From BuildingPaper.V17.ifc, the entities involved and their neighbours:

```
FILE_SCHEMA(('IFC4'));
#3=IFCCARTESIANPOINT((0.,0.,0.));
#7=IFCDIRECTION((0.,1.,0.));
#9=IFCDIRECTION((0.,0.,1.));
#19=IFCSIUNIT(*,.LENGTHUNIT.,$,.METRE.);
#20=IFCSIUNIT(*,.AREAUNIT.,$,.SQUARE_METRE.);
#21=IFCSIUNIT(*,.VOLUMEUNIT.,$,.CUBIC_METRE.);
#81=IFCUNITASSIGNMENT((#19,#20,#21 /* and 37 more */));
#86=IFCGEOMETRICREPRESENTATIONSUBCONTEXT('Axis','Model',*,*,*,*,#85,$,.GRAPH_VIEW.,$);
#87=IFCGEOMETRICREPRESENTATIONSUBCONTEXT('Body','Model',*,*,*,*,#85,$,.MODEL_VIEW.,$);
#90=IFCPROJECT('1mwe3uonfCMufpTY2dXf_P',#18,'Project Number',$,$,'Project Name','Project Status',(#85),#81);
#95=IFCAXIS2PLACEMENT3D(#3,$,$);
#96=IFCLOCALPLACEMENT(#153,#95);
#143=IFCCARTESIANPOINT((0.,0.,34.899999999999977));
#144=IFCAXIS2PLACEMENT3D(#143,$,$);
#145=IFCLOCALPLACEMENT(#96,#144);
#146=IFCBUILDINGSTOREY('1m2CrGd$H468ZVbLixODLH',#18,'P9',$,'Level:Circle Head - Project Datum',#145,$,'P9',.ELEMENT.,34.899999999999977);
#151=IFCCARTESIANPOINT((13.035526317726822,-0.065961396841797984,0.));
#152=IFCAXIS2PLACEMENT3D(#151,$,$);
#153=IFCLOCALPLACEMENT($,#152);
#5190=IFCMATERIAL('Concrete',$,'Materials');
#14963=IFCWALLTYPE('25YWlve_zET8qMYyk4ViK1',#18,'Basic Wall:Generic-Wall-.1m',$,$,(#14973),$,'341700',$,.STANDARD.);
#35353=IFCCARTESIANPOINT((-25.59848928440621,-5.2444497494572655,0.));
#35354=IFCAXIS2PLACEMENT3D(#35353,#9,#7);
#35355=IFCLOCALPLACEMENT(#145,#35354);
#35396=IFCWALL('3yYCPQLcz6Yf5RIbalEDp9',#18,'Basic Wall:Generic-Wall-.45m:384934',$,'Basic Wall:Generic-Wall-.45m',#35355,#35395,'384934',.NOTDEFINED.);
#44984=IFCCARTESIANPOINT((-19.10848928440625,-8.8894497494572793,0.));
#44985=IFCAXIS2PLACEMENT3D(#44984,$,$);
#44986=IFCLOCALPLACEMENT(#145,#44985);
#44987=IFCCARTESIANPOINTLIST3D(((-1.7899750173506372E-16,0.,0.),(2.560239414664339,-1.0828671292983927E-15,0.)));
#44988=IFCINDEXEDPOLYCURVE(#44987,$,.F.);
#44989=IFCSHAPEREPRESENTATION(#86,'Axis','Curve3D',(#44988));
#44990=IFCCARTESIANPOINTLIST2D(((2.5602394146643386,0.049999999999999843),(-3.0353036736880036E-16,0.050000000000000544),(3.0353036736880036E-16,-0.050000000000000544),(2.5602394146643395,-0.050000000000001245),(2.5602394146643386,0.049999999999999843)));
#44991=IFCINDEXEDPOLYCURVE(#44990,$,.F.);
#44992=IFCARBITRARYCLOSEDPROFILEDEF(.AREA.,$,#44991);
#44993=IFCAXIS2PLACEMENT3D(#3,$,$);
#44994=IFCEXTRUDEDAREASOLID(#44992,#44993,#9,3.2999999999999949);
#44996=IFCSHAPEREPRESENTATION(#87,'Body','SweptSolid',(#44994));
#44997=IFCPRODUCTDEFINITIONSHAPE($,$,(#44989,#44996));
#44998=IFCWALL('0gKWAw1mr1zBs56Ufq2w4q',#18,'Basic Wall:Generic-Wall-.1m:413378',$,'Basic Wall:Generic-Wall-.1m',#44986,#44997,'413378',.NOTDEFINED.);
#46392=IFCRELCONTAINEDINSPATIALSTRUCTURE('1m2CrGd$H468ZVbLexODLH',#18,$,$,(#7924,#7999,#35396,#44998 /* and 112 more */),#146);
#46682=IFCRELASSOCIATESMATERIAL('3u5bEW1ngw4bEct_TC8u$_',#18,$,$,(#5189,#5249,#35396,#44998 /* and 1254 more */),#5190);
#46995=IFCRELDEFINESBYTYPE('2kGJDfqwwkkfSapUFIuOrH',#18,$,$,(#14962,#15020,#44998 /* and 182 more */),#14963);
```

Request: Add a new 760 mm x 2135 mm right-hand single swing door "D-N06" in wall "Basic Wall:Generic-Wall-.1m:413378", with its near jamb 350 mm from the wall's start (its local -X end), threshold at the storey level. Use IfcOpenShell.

```python
import numpy as np
import ifcopenshell
import ifcopenshell.api.feature
import ifcopenshell.api.geometry
import ifcopenshell.api.root
import ifcopenshell.api.spatial
import ifcopenshell.geom
import ifcopenshell.util.element
import ifcopenshell.util.placement
import ifcopenshell.util.representation
import ifcopenshell.util.shape
import ifcopenshell.util.unit

model = ifcopenshell.open("BuildingPaper.V17.ifc")
unit_scale = ifcopenshell.util.unit.calculate_unit_scale(model)
settings = ifcopenshell.geom.settings()


def volume(element):
    """Net volume in cubic metres, openings subtracted."""
    shape = ifcopenshell.geom.create_shape(settings, element)
    return ifcopenshell.util.shape.get_volume(shape.geometry)


wall = model.by_guid("0gKWAw1mr1zBs56Ufq2w4q")
storey = ifcopenshell.util.element.get_container(wall, ifc_class="IfcBuildingStorey")
context = ifcopenshell.util.representation.get_context(model, "Model", "Body", "MODEL_VIEW")
before = volume(wall)

width, height, from_end, sill = 0.76, 2.135, 0.35, 0.0  # metres

# The wall runs along its own X axis, and the end named is its -X end.
wall_shape = ifcopenshell.geom.create_shape(settings, wall)
x, y, z = ifcopenshell.util.shape.get_vertices(wall_shape.geometry).T
start = x.min() + from_end
face, thickness = float(y.min()), float(y.max() - y.min())
wall_matrix = ifcopenshell.util.placement.get_local_placement(wall.ObjectPlacement)
level = ifcopenshell.util.placement.get_local_placement(storey.ObjectPlacement)[2, 3]


def in_wall(x, y):
    """Placement at x, y metres in the wall's axes, at sill height."""
    matrix = wall_matrix.copy()
    matrix[:, 3] = wall_matrix @ np.array([x / unit_scale, y / unit_scale, 0.0, 1.0])
    matrix[2, 3] = level + sill / unit_scale
    return matrix


# Opening: a box that overshoots both wall faces by 50 mm.
opening = ifcopenshell.api.root.create_entity(model, ifc_class="IfcOpeningElement", predefined_type="OPENING")
box = ifcopenshell.api.geometry.add_wall_representation(
    model, context=context, length=width, height=height, thickness=thickness + 0.1
)
ifcopenshell.api.geometry.assign_representation(model, product=opening, representation=box)
ifcopenshell.api.geometry.edit_object_placement(model, product=opening, matrix=in_wall(start, face - 0.05), is_si=False)
ifcopenshell.api.feature.add_feature(model, feature=opening, element=wall)

door = ifcopenshell.api.root.create_entity(model, ifc_class="IfcDoor", name="D-N06", predefined_type="DOOR")
door.OverallWidth, door.OverallHeight = width / unit_scale, height / unit_scale
door.OperationType = "SINGLE_SWING_RIGHT"
body = ifcopenshell.api.geometry.add_door_representation(
    model,
    context=context,
    overall_width=door.OverallWidth,
    overall_height=door.OverallHeight,
    operation_type="SINGLE_SWING_RIGHT",
    lining_properties={"LiningDepth": thickness / unit_scale, "ThresholdDepth": thickness / unit_scale},
)
ifcopenshell.api.geometry.assign_representation(model, product=door, representation=body)
ifcopenshell.api.spatial.assign_container(model, products=[door], relating_structure=storey)
ifcopenshell.api.feature.add_filling(model, opening=opening, element=door)

# The lining spans the wall, so the door starts at the wall face.
ifcopenshell.api.geometry.edit_object_placement(model, product=door, matrix=in_wall(start, face), is_si=False)

after = volume(wall)

print(f"wall volume {before:.3f} -> {after:.3f} m3")

model.write("BuildingPaper.V17_updated.ifc")
```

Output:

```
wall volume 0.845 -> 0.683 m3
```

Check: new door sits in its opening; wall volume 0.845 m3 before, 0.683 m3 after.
